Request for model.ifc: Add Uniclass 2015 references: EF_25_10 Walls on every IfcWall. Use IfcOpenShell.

First a look at what the model holds.

```python
import ifcopenshell

model = ifcopenshell.open("model.ifc")
print(model.schema)
print("classifications:", [c.Name for c in model.by_type("IfcClassification")])
for ifc_class in ("IfcDoor", "IfcRoof", "IfcStair", "IfcWall", "IfcWindow"):
    print(ifc_class, len(model.by_type(ifc_class)))
```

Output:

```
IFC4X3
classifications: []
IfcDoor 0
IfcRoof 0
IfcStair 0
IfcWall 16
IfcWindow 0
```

```python
import ifcopenshell
import ifcopenshell.api.classification

model = ifcopenshell.open("model.ifc")

system = ifcopenshell.api.classification.add_classification(model, classification="Uniclass 2015")

codes = {
    "IfcWall": ("EF_25_10", "Walls"),
}
for ifc_class, (code, name) in codes.items():
    products = model.by_type(ifc_class)
    ifcopenshell.api.classification.add_reference(
        model, products=products, classification=system, identification=code, name=name
    )
    print(code, len(products))

model.write("model-out.ifc")
```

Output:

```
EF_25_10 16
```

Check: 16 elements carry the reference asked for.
